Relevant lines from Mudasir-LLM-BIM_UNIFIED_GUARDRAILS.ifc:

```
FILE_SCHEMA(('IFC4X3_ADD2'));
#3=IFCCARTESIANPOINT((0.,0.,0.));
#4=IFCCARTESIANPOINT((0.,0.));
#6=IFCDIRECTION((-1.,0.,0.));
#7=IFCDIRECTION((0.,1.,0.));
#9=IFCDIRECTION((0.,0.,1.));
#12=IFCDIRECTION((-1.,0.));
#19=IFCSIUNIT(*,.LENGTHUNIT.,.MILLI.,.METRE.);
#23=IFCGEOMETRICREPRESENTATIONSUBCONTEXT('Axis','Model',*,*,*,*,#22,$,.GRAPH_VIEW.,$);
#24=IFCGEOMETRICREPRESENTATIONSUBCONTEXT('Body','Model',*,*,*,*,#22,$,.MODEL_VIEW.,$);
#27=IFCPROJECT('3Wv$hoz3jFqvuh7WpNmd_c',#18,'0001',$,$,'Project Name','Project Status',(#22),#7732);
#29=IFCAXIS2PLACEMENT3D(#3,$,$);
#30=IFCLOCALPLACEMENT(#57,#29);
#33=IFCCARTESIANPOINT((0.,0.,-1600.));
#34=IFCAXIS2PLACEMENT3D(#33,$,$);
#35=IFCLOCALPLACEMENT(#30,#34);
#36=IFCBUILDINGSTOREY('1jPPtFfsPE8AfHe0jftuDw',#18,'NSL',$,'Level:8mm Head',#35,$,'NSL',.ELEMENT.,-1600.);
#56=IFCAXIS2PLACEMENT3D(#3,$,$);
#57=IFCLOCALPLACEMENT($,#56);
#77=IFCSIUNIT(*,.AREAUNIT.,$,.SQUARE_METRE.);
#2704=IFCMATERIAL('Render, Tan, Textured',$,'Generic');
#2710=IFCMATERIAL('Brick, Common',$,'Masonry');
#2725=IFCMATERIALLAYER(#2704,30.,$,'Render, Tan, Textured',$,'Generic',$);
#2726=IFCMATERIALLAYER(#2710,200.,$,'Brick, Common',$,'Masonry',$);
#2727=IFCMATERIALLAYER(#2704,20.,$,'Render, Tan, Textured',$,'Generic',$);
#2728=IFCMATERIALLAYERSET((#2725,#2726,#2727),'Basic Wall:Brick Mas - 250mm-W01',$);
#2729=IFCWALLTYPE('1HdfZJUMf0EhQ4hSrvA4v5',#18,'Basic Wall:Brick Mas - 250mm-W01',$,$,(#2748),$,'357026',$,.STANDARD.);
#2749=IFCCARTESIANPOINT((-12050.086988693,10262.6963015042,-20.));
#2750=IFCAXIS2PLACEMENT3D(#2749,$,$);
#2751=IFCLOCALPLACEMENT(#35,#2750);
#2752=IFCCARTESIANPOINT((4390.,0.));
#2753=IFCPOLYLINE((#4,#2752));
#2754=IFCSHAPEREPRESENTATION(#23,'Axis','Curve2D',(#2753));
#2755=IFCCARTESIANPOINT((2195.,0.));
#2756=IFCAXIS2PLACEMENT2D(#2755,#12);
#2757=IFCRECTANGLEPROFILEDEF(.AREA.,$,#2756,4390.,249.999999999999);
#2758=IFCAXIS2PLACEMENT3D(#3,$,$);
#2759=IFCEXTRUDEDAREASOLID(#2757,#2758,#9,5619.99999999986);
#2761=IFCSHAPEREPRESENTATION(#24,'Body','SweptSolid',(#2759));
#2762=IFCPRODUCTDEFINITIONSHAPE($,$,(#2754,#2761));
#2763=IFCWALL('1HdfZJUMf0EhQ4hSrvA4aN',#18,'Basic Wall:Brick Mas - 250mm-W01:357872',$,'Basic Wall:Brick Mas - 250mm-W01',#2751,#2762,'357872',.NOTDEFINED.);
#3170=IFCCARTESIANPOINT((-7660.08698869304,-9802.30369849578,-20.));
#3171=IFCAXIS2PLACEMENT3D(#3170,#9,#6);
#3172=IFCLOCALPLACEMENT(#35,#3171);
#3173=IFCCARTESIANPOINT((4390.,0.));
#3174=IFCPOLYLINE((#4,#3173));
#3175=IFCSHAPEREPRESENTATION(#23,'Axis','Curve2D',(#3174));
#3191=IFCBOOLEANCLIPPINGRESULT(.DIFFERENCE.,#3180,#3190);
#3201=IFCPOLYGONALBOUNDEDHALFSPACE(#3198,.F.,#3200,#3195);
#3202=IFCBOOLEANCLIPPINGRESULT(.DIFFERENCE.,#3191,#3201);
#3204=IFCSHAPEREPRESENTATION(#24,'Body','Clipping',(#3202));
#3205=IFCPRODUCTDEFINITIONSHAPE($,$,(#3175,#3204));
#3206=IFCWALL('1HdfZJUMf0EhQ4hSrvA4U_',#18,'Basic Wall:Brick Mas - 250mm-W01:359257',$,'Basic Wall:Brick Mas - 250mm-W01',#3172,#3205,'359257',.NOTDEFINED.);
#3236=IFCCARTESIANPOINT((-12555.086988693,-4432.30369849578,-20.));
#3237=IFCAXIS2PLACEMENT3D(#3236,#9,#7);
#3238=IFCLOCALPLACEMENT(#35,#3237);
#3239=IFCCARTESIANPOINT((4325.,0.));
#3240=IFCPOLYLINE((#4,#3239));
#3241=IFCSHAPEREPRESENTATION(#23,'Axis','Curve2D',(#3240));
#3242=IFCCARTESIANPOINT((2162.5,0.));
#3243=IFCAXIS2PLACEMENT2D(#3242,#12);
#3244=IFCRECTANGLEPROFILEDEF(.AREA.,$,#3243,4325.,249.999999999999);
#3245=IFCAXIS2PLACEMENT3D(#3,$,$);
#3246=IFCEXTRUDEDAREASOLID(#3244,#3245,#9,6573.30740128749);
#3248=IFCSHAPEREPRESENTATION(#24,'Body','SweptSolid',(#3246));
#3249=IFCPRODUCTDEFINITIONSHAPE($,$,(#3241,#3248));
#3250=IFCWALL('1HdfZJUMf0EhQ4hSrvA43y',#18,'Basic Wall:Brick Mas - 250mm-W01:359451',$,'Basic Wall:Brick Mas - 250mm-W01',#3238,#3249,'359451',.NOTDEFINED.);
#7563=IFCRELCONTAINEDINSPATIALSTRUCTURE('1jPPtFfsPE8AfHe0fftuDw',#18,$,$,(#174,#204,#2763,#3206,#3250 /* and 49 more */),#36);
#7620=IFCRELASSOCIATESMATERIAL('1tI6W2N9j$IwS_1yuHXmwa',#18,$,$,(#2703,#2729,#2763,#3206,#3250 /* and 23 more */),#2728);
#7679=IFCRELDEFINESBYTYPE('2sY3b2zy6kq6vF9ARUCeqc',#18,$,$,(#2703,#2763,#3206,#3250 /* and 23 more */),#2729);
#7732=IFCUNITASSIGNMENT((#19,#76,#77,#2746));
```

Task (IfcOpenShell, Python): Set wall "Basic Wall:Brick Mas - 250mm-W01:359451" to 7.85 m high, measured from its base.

```python
import ifcopenshell
import ifcopenshell.geom
import ifcopenshell.util.representation
import ifcopenshell.util.shape
import ifcopenshell.util.unit

model = ifcopenshell.open("Mudasir-LLM-BIM_UNIFIED_GUARDRAILS.ifc")
unit_scale = ifcopenshell.util.unit.calculate_unit_scale(model)
settings = ifcopenshell.geom.settings()


def volume(element):
    """Net volume in cubic metres, openings subtracted."""
    shape = ifcopenshell.geom.create_shape(settings, element)
    return ifcopenshell.util.shape.get_volume(shape.geometry)


wall = model.by_id(3250)
before = volume(wall)

body = ifcopenshell.util.representation.get_representation(wall, "Model", "Body")
solid = body.Items[0]
old_height = solid.Depth
solid.Depth = 7.85 / unit_scale
after = volume(wall)

print(f"height {old_height:g} -> {solid.Depth:g}, volume {before:.3f} -> {after:.3f} m3")

model.write("Mudasir-LLM-BIM_UNIFIED_GUARDRAILS-out.ifc")
```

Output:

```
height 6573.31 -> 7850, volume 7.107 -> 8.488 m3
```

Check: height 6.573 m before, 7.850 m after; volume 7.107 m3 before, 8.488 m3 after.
